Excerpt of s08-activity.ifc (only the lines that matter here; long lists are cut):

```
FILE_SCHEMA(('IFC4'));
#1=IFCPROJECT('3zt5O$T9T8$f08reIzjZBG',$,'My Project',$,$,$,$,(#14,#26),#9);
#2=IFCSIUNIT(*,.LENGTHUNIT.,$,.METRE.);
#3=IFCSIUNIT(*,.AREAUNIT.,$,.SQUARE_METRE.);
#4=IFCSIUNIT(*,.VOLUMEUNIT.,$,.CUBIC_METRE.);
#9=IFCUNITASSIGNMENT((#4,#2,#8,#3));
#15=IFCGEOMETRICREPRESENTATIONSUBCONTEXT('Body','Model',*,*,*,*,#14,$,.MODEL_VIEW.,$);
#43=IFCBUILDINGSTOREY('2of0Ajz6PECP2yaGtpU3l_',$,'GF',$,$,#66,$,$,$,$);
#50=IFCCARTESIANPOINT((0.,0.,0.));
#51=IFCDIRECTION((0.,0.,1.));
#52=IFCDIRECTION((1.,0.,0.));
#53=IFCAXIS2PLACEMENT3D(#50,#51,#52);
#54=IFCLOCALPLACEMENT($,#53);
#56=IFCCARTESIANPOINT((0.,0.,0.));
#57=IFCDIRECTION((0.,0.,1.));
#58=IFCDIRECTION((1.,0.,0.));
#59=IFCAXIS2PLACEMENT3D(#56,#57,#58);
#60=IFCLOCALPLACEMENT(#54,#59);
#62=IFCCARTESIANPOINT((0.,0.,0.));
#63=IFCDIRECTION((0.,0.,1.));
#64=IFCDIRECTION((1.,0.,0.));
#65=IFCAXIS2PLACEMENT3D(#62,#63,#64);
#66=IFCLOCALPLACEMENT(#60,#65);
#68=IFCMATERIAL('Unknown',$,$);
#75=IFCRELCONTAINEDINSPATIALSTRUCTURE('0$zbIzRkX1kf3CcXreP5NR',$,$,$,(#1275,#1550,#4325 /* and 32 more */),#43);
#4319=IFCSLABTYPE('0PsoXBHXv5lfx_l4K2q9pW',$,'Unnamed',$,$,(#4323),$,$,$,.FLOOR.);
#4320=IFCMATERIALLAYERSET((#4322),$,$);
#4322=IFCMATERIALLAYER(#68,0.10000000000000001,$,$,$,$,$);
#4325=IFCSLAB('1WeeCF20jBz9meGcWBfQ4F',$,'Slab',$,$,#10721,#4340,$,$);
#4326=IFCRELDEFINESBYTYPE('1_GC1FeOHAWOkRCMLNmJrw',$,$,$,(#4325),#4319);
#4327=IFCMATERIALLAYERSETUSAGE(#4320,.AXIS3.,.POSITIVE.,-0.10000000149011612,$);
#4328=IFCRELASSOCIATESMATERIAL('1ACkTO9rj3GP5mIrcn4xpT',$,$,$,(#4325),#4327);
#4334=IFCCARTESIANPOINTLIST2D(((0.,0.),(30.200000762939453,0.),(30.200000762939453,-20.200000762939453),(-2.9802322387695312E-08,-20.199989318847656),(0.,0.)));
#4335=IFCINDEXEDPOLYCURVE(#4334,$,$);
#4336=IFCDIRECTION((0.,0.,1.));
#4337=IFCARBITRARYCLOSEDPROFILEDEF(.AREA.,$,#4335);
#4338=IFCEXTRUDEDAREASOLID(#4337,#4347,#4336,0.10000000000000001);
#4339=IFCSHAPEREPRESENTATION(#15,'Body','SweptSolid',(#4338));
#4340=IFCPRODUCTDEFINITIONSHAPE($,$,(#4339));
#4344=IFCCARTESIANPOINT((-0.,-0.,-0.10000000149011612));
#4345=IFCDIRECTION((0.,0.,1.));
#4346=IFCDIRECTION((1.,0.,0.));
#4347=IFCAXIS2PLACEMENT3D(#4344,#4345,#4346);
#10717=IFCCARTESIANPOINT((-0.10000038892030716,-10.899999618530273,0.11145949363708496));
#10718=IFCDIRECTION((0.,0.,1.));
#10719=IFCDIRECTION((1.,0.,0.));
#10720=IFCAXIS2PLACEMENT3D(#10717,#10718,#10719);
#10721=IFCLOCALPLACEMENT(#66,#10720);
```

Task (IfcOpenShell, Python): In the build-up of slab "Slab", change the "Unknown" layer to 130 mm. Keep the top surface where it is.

```python
import ifcopenshell
import ifcopenshell.util.element
import ifcopenshell.util.representation
import ifcopenshell.util.unit

model = ifcopenshell.open("s08-activity.ifc")
unit_scale = ifcopenshell.util.unit.calculate_unit_scale(model)

layer_set = model.by_id(4320)
layer = next(l for l in layer_set.MaterialLayers if l.Material and l.Material.Name == "Unknown")
change = 0.13 / unit_scale - layer.LayerThickness
layer.LayerThickness += change

# Geometry does not follow the layer set by itself.
slabs = [e for e in ifcopenshell.util.element.get_elements_by_material(model, layer_set) if e.is_a("IfcSlab")]
for slab in sorted(slabs, key=lambda e: e.id()):
    body = ifcopenshell.util.representation.get_representation(slab, "Model", "Body")
    solid = body.Items[0]
    old_depth = solid.Depth
    solid.Depth += change
    # Extruded upwards: lower the start of the extrusion so the top stays.
    x, y, z = solid.Position.Location.Coordinates
    solid.Position.Location = model.createIfcCartesianPoint((x, y, z - change))
    print(slab.id(), f"{old_depth:g} -> {solid.Depth:g}")

# The layers are counted up from the underside, which has moved.
for usage in {ifcopenshell.util.element.get_material(slab) for slab in slabs}:
    usage.OffsetFromReferenceLine -= change

model.write("s08-activity-out.ifc")
```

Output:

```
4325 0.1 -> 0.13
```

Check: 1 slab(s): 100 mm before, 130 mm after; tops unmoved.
